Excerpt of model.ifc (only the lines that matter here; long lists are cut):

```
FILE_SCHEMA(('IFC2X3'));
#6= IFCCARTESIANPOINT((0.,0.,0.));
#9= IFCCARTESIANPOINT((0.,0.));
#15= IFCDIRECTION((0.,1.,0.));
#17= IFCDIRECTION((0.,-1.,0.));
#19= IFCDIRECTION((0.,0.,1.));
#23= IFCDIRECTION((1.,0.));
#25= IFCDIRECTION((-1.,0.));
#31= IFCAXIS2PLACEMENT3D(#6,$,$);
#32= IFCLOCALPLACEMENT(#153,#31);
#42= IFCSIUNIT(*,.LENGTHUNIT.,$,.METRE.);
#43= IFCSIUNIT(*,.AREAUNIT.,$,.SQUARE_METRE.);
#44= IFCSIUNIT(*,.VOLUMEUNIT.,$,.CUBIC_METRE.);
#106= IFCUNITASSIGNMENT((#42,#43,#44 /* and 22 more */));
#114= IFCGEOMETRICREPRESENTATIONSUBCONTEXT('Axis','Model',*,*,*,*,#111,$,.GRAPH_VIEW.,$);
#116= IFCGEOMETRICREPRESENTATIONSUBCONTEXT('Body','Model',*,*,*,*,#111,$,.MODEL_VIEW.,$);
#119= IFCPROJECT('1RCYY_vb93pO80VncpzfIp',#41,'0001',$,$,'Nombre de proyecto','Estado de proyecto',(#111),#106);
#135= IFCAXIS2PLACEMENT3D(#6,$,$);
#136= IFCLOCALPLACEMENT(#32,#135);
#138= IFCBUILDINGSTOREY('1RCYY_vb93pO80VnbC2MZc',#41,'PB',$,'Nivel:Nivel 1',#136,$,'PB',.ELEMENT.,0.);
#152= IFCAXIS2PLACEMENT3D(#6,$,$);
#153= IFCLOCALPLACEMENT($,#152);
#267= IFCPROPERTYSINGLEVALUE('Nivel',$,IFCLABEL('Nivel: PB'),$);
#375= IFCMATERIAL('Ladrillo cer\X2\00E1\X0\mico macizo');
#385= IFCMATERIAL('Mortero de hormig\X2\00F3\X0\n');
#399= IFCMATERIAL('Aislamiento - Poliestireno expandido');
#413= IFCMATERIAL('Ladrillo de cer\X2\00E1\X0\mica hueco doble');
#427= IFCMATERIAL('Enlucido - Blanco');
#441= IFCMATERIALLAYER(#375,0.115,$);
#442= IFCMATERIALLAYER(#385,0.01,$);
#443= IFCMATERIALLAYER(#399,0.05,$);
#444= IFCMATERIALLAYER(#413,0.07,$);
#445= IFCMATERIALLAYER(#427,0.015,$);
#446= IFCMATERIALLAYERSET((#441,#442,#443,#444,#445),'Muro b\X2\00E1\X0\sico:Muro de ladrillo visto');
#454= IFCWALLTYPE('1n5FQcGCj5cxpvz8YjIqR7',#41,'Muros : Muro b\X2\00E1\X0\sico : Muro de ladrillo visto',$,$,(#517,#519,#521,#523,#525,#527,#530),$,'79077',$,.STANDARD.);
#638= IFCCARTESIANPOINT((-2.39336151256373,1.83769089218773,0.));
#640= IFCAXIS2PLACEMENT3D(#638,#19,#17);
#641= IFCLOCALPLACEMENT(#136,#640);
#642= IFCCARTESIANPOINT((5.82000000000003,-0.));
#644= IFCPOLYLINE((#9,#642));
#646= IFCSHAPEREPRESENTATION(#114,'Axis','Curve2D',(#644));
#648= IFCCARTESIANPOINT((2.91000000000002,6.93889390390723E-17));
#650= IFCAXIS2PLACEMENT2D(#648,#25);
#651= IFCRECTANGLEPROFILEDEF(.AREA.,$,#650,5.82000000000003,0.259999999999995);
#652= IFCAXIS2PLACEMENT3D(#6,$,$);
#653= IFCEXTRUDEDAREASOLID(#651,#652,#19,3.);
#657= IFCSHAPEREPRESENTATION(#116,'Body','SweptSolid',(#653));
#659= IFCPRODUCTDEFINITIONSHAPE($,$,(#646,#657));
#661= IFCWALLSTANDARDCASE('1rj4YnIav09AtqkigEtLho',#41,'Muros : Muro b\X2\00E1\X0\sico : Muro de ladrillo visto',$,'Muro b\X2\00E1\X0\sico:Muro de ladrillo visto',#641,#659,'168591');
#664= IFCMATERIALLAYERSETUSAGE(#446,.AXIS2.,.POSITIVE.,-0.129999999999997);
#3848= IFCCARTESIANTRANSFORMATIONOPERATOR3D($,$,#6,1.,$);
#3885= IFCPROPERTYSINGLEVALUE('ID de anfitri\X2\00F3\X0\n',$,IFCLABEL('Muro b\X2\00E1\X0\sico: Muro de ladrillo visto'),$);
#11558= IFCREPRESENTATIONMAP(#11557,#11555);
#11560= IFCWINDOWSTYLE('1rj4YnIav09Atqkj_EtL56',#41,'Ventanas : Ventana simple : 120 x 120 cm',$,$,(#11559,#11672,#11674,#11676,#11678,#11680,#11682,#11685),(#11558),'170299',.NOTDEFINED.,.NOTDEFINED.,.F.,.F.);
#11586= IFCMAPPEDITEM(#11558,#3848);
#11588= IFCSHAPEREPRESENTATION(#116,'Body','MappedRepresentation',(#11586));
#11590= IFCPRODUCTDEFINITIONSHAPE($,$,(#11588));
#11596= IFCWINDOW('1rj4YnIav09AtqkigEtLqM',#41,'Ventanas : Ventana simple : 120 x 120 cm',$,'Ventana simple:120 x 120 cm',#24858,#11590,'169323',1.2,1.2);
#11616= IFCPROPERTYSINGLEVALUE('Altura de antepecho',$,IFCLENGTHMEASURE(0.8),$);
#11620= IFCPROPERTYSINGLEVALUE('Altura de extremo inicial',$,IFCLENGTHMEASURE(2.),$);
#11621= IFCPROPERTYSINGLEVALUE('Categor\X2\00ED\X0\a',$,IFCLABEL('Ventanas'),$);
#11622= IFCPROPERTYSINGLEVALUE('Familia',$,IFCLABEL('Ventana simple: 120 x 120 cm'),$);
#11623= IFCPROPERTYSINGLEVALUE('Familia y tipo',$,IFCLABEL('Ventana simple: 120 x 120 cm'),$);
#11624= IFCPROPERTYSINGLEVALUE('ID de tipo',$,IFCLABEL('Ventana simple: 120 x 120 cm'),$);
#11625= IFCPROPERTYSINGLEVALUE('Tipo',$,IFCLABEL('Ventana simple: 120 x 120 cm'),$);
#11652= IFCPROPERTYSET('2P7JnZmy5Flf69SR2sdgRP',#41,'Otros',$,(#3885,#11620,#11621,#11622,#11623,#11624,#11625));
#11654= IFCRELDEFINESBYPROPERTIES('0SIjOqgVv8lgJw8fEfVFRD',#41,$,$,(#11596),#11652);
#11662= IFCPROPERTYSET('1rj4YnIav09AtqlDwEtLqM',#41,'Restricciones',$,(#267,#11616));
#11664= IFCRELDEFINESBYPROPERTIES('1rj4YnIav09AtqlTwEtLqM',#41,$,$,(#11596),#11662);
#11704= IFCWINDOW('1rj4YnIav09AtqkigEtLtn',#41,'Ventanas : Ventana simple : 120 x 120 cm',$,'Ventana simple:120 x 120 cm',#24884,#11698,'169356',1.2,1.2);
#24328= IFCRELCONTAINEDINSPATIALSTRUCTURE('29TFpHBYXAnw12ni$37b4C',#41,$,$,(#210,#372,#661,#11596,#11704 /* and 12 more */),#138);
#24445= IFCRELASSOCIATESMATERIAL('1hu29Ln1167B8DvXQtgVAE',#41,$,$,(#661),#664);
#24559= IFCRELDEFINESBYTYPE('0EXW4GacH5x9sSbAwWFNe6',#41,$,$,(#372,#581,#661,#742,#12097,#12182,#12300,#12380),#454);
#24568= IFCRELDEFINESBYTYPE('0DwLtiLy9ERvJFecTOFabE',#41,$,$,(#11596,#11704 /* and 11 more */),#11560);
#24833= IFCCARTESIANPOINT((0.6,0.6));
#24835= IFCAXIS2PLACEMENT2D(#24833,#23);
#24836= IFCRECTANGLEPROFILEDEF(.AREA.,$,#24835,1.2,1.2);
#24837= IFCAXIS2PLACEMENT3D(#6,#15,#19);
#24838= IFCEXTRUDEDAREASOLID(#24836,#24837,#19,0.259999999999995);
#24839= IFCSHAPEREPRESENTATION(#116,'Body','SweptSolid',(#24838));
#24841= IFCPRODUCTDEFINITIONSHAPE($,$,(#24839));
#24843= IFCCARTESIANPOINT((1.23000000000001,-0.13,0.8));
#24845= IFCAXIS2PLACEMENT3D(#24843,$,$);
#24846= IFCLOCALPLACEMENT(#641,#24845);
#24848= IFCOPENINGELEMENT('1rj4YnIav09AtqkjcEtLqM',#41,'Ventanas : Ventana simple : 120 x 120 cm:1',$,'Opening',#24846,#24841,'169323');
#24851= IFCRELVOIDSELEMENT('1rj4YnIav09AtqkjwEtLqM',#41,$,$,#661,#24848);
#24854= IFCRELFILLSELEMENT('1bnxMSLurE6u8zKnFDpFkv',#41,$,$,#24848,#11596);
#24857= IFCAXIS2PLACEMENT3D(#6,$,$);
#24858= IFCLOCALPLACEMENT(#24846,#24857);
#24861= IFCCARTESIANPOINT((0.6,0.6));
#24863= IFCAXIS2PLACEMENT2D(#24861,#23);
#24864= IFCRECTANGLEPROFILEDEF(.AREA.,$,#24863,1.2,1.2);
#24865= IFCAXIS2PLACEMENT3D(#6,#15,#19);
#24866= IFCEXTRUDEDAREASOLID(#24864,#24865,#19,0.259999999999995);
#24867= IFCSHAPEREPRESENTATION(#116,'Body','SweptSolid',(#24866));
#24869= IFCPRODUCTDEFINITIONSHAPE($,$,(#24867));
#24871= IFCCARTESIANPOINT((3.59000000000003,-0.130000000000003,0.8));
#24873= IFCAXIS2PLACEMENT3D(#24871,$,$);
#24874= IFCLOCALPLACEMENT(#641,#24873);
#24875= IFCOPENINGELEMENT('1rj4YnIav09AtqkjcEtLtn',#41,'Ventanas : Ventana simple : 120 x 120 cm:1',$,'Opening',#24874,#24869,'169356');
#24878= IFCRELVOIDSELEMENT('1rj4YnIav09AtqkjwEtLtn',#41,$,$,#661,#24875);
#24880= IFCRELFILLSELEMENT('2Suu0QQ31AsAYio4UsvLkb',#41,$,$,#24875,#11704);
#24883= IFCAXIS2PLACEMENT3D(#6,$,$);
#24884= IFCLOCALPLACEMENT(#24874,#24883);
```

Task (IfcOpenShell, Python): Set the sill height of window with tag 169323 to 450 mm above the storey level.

```python
import numpy as np
import ifcopenshell
import ifcopenshell.api.geometry
import ifcopenshell.api.pset
import ifcopenshell.geom
import ifcopenshell.util.element
import ifcopenshell.util.placement
import ifcopenshell.util.shape
import ifcopenshell.util.unit

model = ifcopenshell.open("model.ifc")
unit_scale = ifcopenshell.util.unit.calculate_unit_scale(model)

window = model.by_guid("1rj4YnIav09AtqkigEtLqM")
opening = window.FillsVoids[0].RelatingOpeningElement
storey = ifcopenshell.util.element.get_container(window, ifc_class="IfcBuildingStorey")
level = ifcopenshell.util.placement.get_local_placement(storey.ObjectPlacement)[2, 3]

# The opening's origin need not be at the sill, so measure its lowest point.
shape = ifcopenshell.geom.create_shape(ifcopenshell.geom.settings(), opening)
bottom = ifcopenshell.util.shape.get_shape_bottom_elevation(shape, shape.geometry) / unit_scale
dz = level + 0.45 - bottom

shift = np.array([0.0, 0.0, dz])
# The window is placed relative to its opening, so it follows when the opening moves.
matrix = ifcopenshell.util.placement.get_local_placement(opening.ObjectPlacement)
matrix[:3, 3] += shift
ifcopenshell.api.geometry.edit_object_placement(
    model, product=opening, matrix=matrix, is_si=False, should_transform_children=True
)

# Keep the stored heights in step.
pset = model.by_id(ifcopenshell.util.element.get_pset(window, "Otros", should_inherit=False)["id"])
ifcopenshell.api.pset.edit_pset(model, pset=pset, properties={
    "Altura de extremo inicial": model.create_entity("IfcLengthMeasure", ifcopenshell.util.element.get_pset(window, "Otros", "Altura de extremo inicial") + dz),
})
pset = model.by_id(ifcopenshell.util.element.get_pset(window, "Restricciones", should_inherit=False)["id"])
ifcopenshell.api.pset.edit_pset(model, pset=pset, properties={
    "Altura de antepecho": model.create_entity("IfcLengthMeasure", ifcopenshell.util.element.get_pset(window, "Restricciones", "Altura de antepecho") + dz),
})

print(f"moved by {dz * unit_scale:+.3f} m")

model.write("model_rev.ifc")
```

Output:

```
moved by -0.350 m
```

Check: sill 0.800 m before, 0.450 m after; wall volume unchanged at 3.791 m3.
